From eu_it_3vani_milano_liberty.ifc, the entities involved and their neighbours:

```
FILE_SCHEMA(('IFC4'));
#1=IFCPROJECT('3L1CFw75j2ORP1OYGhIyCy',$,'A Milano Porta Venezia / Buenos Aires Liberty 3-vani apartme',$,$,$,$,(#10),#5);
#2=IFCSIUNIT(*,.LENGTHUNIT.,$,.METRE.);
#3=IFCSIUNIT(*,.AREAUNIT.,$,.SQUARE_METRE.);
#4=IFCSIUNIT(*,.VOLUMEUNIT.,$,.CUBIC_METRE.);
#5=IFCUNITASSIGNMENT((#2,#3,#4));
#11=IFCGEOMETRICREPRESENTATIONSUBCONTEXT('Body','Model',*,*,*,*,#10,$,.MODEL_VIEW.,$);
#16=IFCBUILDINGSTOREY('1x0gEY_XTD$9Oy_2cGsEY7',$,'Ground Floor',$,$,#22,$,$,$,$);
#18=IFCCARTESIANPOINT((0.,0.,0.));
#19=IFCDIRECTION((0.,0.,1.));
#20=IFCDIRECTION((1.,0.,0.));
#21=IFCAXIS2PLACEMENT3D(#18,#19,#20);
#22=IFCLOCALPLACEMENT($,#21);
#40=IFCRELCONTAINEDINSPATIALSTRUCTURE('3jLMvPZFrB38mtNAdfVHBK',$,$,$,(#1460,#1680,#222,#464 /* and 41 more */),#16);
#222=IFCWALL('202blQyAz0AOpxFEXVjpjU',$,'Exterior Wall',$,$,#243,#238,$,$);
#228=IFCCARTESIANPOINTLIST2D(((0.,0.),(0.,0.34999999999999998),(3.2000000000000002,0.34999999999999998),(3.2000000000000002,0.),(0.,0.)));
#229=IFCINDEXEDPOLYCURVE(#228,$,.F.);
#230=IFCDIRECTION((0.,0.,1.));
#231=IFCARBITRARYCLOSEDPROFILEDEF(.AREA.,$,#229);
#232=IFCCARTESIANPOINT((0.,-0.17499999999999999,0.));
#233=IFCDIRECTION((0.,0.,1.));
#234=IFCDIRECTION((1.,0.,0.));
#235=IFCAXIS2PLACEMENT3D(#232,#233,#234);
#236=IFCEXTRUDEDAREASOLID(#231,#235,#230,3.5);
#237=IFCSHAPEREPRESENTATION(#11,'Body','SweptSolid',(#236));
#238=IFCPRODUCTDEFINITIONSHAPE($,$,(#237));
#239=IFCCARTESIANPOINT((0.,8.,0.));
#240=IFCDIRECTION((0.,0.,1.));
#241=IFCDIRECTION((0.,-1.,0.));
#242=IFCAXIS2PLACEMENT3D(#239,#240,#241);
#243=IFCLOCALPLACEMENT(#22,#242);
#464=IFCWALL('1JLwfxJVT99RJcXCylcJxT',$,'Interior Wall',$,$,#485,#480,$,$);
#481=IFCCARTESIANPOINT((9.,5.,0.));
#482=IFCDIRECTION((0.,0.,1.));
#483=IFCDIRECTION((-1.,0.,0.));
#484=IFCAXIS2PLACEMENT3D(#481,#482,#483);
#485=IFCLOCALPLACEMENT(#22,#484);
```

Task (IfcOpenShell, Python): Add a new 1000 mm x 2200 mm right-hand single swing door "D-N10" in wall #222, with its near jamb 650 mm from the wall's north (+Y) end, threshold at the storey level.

```python
import numpy as np
import ifcopenshell
import ifcopenshell.api.feature
import ifcopenshell.api.geometry
import ifcopenshell.api.root
import ifcopenshell.api.spatial
import ifcopenshell.geom
import ifcopenshell.util.element
import ifcopenshell.util.placement
import ifcopenshell.util.representation
import ifcopenshell.util.shape
import ifcopenshell.util.unit

model = ifcopenshell.open("eu_it_3vani_milano_liberty.ifc")
unit_scale = ifcopenshell.util.unit.calculate_unit_scale(model)
settings = ifcopenshell.geom.settings()


def volume(element):
    """Net volume in cubic metres, openings subtracted."""
    shape = ifcopenshell.geom.create_shape(settings, element)
    return ifcopenshell.util.shape.get_volume(shape.geometry)


wall = model.by_id(222)
storey = ifcopenshell.util.element.get_container(wall, ifc_class="IfcBuildingStorey")
context = ifcopenshell.util.representation.get_context(model, "Model", "Body", "MODEL_VIEW")
before = volume(wall)

width, height, from_end, sill = 1, 2.2, 0.65, 0.0  # metres

# The wall runs along its own X axis, and the end named is its -X end.
wall_shape = ifcopenshell.geom.create_shape(settings, wall)
x, y, z = ifcopenshell.util.shape.get_vertices(wall_shape.geometry).T
start = x.min() + from_end
face, thickness = float(y.min()), float(y.max() - y.min())
wall_matrix = ifcopenshell.util.placement.get_local_placement(wall.ObjectPlacement)
level = ifcopenshell.util.placement.get_local_placement(storey.ObjectPlacement)[2, 3]


def in_wall(x, y):
    """Placement at x, y metres in the wall's axes, at sill height."""
    matrix = wall_matrix.copy()
    matrix[:, 3] = wall_matrix @ np.array([x / unit_scale, y / unit_scale, 0.0, 1.0])
    matrix[2, 3] = level + sill / unit_scale
    return matrix


# Opening: a box that overshoots both wall faces by 50 mm.
opening = ifcopenshell.api.root.create_entity(model, ifc_class="IfcOpeningElement", predefined_type="OPENING")
box = ifcopenshell.api.geometry.add_wall_representation(
    model, context=context, length=width, height=height, thickness=thickness + 0.1
)
ifcopenshell.api.geometry.assign_representation(model, product=opening, representation=box)
ifcopenshell.api.geometry.edit_object_placement(model, product=opening, matrix=in_wall(start, face - 0.05), is_si=False)
ifcopenshell.api.feature.add_feature(model, feature=opening, element=wall)

door = ifcopenshell.api.root.create_entity(model, ifc_class="IfcDoor", name="D-N10", predefined_type="DOOR")
door.OverallWidth, door.OverallHeight = width / unit_scale, height / unit_scale
door.OperationType = "SINGLE_SWING_RIGHT"
body = ifcopenshell.api.geometry.add_door_representation(
    model,
    context=context,
    overall_width=door.OverallWidth,
    overall_height=door.OverallHeight,
    operation_type="SINGLE_SWING_RIGHT",
    lining_properties={"LiningDepth": thickness / unit_scale, "ThresholdDepth": thickness / unit_scale},
)
ifcopenshell.api.geometry.assign_representation(model, product=door, representation=body)
ifcopenshell.api.spatial.assign_container(model, products=[door], relating_structure=storey)
ifcopenshell.api.feature.add_filling(model, opening=opening, element=door)

# The lining spans the wall, so the door starts at the wall face.
ifcopenshell.api.geometry.edit_object_placement(model, product=door, matrix=in_wall(start, face), is_si=False)

after = volume(wall)

print(f"wall volume {before:.3f} -> {after:.3f} m3")

model.write("eu_it_3vani_milano_liberty_updated.ifc")
```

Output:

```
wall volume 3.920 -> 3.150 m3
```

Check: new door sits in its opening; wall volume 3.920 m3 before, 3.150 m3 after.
